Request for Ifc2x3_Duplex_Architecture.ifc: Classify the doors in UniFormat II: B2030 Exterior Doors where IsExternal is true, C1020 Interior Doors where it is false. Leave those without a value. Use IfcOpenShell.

First a look at what the model holds.

```python
import ifcopenshell
import ifcopenshell.util.element

model = ifcopenshell.open("Ifc2x3_Duplex_Architecture.ifc")
print(model.schema)
print("classifications:", [c.Name for c in model.by_type("IfcClassification")])
values = [ifcopenshell.util.element.get_pset(e, "Pset_DoorCommon", "IsExternal") for e in model.by_type("IfcDoor")]
for value in (True, False, None):
    print("IsExternal", value, values.count(value))
```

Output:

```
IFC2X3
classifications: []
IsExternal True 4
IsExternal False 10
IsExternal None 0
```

```python
import ifcopenshell
import ifcopenshell.api.classification
import ifcopenshell.util.element

model = ifcopenshell.open("Ifc2x3_Duplex_Architecture.ifc")

# IFC2X3 requires Source and Edition and has no link from the project to the system.
system = model.create_entity("IfcClassification", Source="ASTM", Edition="E1557", Name="UniFormat II")

doors = model.by_type("IfcDoor")
external = {e: ifcopenshell.util.element.get_pset(e, "Pset_DoorCommon", "IsExternal") for e in doors}
for flag, code, name in ((True, "B2030", "Exterior Doors"), (False, "C1020", "Interior Doors")):
    products = [e for e in doors if external[e] is flag]
    ifcopenshell.api.classification.add_reference(
        model, products=products, classification=system, identification=code, name=name
    )
    print(code, len(products))

model.write("Ifc2x3_Duplex_Architecture-out.ifc")
```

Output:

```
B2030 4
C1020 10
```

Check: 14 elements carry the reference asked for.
